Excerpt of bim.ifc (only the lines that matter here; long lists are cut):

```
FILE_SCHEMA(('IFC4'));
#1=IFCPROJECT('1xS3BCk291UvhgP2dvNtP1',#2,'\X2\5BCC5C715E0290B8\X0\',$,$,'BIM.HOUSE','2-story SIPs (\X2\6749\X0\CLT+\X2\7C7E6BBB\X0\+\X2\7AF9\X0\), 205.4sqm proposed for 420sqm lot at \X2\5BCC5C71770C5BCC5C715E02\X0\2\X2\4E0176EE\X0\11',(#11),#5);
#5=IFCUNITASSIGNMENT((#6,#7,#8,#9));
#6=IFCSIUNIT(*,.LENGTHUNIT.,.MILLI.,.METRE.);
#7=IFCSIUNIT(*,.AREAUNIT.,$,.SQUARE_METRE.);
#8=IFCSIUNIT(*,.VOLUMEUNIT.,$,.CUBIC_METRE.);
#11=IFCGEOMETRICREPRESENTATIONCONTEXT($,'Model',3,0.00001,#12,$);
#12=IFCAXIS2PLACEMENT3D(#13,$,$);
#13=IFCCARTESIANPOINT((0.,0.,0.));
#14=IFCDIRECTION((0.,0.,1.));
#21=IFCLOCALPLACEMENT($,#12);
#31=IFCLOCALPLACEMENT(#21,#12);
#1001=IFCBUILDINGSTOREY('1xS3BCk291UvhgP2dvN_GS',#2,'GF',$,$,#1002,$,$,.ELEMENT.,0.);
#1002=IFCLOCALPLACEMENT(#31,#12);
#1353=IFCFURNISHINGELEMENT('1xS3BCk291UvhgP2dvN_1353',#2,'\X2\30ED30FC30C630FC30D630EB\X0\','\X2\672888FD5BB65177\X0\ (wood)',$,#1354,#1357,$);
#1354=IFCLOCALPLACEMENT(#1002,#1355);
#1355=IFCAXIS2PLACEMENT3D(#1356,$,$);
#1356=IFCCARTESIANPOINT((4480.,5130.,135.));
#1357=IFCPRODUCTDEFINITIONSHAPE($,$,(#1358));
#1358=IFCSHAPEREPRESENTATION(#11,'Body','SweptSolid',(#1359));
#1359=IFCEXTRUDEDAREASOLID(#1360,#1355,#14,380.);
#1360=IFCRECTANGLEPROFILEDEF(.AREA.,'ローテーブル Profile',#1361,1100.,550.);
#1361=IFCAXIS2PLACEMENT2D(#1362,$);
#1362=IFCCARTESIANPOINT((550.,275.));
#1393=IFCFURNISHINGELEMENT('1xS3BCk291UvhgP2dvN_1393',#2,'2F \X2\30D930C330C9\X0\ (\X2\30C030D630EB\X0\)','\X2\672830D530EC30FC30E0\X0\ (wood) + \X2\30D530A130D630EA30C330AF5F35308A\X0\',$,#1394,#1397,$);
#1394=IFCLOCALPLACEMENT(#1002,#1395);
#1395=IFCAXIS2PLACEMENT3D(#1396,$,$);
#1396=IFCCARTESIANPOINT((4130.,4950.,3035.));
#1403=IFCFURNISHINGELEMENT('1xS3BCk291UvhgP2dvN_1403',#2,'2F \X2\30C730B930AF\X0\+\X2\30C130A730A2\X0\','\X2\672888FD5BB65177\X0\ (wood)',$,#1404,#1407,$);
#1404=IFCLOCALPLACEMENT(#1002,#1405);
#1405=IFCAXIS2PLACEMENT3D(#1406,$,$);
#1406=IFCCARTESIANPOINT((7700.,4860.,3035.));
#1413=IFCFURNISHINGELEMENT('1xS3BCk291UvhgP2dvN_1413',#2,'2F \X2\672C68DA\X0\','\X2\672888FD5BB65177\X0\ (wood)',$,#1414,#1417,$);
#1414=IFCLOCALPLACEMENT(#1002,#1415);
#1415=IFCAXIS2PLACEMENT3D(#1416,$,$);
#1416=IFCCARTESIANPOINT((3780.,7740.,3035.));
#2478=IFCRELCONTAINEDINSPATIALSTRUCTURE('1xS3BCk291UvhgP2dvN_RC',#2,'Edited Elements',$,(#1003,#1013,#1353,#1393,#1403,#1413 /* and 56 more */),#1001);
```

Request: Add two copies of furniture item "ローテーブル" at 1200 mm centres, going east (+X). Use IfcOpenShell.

```python
import numpy as np
import ifcopenshell
import ifcopenshell.api.geometry
import ifcopenshell.api.root
import ifcopenshell.util.element
import ifcopenshell.util.placement
import ifcopenshell.util.unit

model = ifcopenshell.open("bim.ifc")
unit_scale = ifcopenshell.util.unit.calculate_unit_scale(model)


def reuse_history(source, copy):
    """copy_class also copies each property set's owner history, people and application; keep the originals."""
    for rel in copy.IsDefinedBy:
        if rel.is_a("IfcRelDefinesByProperties") and (history := rel.RelatingPropertyDefinition.OwnerHistory):
            rel.RelatingPropertyDefinition.OwnerHistory = source.OwnerHistory
            ifcopenshell.util.element.remove_deep2(model, history)


source = model.by_guid("1xS3BCk291UvhgP2dvN_1353")
base = ifcopenshell.util.placement.get_local_placement(source.ObjectPlacement)
step = np.array([1.0, 0.0, 0.0]) * 1.2 / unit_scale

for i in range(1, 3):
    copy = ifcopenshell.api.root.copy_class(model, product=source)
    copy.Representation = ifcopenshell.util.element.copy_deep(
        model, source.Representation, exclude=["IfcGeometricRepresentationContext", "IfcRepresentationMap"]
    )
    reuse_history(source, copy)
    matrix = base.copy()
    matrix[:3, 3] += i * step
    print("added at", matrix[:3, 3].round(3) + 0.0)
    ifcopenshell.api.geometry.edit_object_placement(model, product=copy, matrix=matrix, is_si=False)

model.write("bim_rev.ifc")
```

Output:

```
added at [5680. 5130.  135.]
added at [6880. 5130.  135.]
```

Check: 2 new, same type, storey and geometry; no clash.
